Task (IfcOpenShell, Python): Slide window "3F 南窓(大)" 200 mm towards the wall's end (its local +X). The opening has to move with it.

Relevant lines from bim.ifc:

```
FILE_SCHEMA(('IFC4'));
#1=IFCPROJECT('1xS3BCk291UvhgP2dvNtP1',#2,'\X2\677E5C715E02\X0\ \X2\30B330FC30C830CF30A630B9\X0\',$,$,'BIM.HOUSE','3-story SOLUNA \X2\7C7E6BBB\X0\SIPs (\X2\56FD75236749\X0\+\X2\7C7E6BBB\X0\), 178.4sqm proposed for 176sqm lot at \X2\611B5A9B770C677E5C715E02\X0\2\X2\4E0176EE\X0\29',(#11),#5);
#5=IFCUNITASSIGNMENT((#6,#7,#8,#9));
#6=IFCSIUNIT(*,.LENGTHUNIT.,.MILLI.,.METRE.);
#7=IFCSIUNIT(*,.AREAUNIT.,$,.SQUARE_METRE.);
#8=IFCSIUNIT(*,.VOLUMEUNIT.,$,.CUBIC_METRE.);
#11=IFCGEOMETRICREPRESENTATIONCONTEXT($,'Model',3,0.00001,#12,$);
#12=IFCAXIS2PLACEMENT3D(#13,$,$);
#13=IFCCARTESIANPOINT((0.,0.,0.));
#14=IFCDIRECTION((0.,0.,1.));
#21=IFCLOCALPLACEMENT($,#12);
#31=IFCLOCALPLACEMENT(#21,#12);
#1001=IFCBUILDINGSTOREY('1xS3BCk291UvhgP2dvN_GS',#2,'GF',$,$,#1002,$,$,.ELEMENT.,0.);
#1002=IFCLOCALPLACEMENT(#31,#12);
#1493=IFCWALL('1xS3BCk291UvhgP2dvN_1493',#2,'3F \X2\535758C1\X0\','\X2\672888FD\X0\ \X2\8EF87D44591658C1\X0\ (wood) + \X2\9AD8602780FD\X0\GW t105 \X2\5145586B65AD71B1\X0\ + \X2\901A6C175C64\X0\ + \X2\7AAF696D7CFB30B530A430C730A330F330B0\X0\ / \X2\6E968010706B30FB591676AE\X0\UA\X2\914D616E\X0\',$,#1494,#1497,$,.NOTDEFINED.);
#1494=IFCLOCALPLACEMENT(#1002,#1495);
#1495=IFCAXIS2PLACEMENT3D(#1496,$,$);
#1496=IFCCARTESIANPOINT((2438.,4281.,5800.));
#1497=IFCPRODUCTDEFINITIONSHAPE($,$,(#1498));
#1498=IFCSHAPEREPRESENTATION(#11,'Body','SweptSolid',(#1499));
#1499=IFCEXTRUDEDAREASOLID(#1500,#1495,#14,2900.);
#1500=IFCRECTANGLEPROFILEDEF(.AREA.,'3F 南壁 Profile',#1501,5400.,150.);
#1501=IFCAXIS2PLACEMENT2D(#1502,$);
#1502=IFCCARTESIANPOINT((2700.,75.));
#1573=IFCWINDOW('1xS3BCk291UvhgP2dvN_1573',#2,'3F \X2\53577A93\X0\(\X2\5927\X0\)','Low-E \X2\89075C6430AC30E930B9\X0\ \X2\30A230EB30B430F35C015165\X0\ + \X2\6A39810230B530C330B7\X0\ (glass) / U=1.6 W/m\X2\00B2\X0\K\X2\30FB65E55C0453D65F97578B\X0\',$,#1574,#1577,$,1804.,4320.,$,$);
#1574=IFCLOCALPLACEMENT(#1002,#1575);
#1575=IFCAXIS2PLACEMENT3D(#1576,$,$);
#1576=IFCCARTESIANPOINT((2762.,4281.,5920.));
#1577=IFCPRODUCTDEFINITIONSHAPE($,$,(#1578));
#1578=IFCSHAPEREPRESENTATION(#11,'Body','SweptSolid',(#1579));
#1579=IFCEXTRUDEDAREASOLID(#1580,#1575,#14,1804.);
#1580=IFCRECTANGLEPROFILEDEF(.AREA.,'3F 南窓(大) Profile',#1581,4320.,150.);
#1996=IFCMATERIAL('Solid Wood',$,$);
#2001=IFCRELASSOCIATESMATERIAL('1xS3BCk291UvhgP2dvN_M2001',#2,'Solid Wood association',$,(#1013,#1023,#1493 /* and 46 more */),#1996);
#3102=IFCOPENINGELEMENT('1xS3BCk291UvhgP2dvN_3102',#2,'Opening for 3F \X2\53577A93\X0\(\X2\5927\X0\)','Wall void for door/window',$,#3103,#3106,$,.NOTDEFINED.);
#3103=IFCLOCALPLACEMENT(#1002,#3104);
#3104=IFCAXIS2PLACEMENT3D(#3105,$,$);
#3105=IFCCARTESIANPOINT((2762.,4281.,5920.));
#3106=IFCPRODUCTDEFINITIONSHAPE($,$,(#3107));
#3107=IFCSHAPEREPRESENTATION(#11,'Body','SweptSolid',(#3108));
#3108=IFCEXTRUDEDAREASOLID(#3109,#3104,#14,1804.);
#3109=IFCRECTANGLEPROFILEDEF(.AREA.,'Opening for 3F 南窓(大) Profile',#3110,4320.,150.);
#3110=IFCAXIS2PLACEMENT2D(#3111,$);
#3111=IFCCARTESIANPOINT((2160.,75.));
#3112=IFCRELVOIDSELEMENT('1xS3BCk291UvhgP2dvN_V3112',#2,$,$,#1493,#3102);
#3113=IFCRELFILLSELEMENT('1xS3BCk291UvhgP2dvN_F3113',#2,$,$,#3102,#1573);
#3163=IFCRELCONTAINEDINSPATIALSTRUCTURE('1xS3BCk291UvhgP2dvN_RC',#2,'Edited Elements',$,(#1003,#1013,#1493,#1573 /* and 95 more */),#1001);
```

```python
import ifcopenshell
import ifcopenshell.api.geometry
import ifcopenshell.util.placement

model = ifcopenshell.open("bim.ifc")

window = model.by_guid("1xS3BCk291UvhgP2dvN_1573")
opening = window.FillsVoids[0].RelatingOpeningElement
wall = opening.VoidsElements[0].RelatingBuildingElement

wall_matrix = ifcopenshell.util.placement.get_local_placement(wall.ObjectPlacement)
shift = wall_matrix[:3, 0] * 200.0
before = ifcopenshell.util.placement.get_local_placement(window.ObjectPlacement)[:3, 3].copy()

# The window is not placed relative to its opening, so move both.
for product in (opening, window):
    matrix = ifcopenshell.util.placement.get_local_placement(product.ObjectPlacement)
    matrix[:3, 3] += shift
    ifcopenshell.api.geometry.edit_object_placement(model, product=product, matrix=matrix, is_si=False)

after = ifcopenshell.util.placement.get_local_placement(window.ObjectPlacement)[:3, 3]
print("window moved by", (after - before).round(3) + 0.0)

model.write("bim_rev.ifc")
```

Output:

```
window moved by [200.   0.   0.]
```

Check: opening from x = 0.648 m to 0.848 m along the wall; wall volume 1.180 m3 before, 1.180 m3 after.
